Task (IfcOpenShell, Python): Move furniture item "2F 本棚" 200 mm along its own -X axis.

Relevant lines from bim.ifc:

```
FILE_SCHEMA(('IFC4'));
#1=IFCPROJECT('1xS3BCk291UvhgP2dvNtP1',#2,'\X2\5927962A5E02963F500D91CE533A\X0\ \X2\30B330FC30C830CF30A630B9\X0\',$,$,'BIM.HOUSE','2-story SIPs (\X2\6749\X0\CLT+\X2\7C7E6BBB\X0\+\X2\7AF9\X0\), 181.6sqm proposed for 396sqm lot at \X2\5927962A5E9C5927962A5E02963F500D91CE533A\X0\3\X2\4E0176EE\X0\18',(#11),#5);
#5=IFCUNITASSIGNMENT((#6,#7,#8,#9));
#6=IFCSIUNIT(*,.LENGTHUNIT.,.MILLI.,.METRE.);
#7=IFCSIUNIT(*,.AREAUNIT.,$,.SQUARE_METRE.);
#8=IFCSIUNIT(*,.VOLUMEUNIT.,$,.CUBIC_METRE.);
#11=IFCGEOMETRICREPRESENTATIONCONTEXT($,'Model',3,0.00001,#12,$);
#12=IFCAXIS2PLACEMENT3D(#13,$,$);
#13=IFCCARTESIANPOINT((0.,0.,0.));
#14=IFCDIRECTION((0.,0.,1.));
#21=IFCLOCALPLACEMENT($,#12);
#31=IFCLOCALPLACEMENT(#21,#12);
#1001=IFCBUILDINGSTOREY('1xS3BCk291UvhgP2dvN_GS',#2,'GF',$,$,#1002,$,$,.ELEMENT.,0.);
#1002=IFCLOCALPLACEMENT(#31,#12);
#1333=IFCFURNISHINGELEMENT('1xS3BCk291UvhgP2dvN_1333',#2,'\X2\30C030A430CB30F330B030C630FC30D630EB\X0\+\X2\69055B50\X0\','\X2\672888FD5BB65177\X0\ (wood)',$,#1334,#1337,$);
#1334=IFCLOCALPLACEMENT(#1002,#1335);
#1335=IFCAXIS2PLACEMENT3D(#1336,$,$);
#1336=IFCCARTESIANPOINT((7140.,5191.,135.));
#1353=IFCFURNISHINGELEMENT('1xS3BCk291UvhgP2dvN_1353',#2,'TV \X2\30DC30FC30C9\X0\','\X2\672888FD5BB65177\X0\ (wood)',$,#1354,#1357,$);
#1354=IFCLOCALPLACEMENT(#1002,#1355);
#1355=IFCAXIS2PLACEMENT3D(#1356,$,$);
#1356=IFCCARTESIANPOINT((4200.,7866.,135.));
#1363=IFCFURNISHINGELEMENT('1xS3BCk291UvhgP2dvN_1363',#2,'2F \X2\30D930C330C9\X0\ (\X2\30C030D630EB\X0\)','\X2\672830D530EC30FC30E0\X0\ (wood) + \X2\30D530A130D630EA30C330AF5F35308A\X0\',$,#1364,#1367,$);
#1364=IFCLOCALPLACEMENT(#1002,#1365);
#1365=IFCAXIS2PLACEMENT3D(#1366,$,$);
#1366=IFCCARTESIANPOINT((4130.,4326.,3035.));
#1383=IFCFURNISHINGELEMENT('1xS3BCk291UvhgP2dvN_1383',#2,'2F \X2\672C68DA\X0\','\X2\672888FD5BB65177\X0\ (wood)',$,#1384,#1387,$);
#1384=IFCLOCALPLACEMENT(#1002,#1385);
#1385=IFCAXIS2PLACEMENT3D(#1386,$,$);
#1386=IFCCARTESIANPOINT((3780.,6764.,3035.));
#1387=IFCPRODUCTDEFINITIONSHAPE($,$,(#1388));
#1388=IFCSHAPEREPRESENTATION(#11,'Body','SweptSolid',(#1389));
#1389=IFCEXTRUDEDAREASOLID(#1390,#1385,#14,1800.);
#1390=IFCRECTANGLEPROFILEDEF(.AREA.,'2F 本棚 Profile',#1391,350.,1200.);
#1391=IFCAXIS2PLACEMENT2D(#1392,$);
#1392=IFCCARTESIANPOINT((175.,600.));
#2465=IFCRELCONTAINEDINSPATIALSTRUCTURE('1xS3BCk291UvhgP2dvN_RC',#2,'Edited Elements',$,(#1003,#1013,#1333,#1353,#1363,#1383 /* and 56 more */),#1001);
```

```python
import ifcopenshell
import ifcopenshell.api.geometry
import ifcopenshell.util.placement
import ifcopenshell.util.unit

model = ifcopenshell.open("bim.ifc")
unit_scale = ifcopenshell.util.unit.calculate_unit_scale(model)

item = model.by_id(1383)
matrix = ifcopenshell.util.placement.get_local_placement(item.ObjectPlacement)
matrix[:3, 3] -= matrix[:3, 0] * 0.2 / unit_scale
ifcopenshell.api.geometry.edit_object_placement(model, product=item, matrix=matrix, is_si=False)

print(ifcopenshell.util.placement.get_local_placement(item.ObjectPlacement).round(3) + 0.0)

model.write("bim_v2.ifc")
```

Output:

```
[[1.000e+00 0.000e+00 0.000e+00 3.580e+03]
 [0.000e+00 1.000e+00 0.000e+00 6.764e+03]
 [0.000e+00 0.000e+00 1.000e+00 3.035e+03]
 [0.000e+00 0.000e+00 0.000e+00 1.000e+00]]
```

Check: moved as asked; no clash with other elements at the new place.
